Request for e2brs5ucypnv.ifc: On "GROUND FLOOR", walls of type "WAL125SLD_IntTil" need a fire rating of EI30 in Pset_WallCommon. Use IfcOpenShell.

First a look at what the model holds.

```python
import ifcopenshell
import ifcopenshell.util.element

model = ifcopenshell.open("e2brs5ucypnv.ifc")
print(model.schema)
storey = next(s for s in model.by_type("IfcBuildingStorey") if s.Name == "GROUND FLOOR")
walls = [e for e in ifcopenshell.util.element.get_decomposition(storey) if e.is_a("IfcWall")]
seen = {}
for e in walls:
    element_type = ifcopenshell.util.element.get_type(e)
    key = (element_type.Name if element_type != e and element_type else None, ifcopenshell.util.element.get_pset(e, "Pset_WallCommon", "FireRating"))
    seen[key] = seen.get(key, 0) + 1
for (name, value), count in sorted(seen.items(), key=str):
    print(count, "x", name, "|", value)
```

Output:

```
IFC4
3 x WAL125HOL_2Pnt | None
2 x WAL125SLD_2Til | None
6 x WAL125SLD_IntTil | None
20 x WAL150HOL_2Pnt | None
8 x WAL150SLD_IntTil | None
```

```python
import ifcopenshell
import ifcopenshell.api.pset
import ifcopenshell.util.element

model = ifcopenshell.open("e2brs5ucypnv.ifc")

storey = next(s for s in model.by_type("IfcBuildingStorey") if s.Name == "GROUND FLOOR")
walls = [e for e in ifcopenshell.util.element.get_decomposition(storey) if e.is_a("IfcWall")]

count = 0
for e in walls:
    element_type = ifcopenshell.util.element.get_type(e)
    if element_type in (None, e) or element_type.Name != "WAL125SLD_IntTil":
        continue
    # add_pset returns the element's existing set when there is one.
    pset = ifcopenshell.api.pset.add_pset(model, product=e, name="Pset_WallCommon")
    ifcopenshell.api.pset.edit_pset(model, pset=pset, properties={"FireRating": "EI30"})
    count += 1

print(count, "walls updated")

model.write("e2brs5ucypnv-out.ifc")
```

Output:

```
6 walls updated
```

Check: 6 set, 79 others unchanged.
